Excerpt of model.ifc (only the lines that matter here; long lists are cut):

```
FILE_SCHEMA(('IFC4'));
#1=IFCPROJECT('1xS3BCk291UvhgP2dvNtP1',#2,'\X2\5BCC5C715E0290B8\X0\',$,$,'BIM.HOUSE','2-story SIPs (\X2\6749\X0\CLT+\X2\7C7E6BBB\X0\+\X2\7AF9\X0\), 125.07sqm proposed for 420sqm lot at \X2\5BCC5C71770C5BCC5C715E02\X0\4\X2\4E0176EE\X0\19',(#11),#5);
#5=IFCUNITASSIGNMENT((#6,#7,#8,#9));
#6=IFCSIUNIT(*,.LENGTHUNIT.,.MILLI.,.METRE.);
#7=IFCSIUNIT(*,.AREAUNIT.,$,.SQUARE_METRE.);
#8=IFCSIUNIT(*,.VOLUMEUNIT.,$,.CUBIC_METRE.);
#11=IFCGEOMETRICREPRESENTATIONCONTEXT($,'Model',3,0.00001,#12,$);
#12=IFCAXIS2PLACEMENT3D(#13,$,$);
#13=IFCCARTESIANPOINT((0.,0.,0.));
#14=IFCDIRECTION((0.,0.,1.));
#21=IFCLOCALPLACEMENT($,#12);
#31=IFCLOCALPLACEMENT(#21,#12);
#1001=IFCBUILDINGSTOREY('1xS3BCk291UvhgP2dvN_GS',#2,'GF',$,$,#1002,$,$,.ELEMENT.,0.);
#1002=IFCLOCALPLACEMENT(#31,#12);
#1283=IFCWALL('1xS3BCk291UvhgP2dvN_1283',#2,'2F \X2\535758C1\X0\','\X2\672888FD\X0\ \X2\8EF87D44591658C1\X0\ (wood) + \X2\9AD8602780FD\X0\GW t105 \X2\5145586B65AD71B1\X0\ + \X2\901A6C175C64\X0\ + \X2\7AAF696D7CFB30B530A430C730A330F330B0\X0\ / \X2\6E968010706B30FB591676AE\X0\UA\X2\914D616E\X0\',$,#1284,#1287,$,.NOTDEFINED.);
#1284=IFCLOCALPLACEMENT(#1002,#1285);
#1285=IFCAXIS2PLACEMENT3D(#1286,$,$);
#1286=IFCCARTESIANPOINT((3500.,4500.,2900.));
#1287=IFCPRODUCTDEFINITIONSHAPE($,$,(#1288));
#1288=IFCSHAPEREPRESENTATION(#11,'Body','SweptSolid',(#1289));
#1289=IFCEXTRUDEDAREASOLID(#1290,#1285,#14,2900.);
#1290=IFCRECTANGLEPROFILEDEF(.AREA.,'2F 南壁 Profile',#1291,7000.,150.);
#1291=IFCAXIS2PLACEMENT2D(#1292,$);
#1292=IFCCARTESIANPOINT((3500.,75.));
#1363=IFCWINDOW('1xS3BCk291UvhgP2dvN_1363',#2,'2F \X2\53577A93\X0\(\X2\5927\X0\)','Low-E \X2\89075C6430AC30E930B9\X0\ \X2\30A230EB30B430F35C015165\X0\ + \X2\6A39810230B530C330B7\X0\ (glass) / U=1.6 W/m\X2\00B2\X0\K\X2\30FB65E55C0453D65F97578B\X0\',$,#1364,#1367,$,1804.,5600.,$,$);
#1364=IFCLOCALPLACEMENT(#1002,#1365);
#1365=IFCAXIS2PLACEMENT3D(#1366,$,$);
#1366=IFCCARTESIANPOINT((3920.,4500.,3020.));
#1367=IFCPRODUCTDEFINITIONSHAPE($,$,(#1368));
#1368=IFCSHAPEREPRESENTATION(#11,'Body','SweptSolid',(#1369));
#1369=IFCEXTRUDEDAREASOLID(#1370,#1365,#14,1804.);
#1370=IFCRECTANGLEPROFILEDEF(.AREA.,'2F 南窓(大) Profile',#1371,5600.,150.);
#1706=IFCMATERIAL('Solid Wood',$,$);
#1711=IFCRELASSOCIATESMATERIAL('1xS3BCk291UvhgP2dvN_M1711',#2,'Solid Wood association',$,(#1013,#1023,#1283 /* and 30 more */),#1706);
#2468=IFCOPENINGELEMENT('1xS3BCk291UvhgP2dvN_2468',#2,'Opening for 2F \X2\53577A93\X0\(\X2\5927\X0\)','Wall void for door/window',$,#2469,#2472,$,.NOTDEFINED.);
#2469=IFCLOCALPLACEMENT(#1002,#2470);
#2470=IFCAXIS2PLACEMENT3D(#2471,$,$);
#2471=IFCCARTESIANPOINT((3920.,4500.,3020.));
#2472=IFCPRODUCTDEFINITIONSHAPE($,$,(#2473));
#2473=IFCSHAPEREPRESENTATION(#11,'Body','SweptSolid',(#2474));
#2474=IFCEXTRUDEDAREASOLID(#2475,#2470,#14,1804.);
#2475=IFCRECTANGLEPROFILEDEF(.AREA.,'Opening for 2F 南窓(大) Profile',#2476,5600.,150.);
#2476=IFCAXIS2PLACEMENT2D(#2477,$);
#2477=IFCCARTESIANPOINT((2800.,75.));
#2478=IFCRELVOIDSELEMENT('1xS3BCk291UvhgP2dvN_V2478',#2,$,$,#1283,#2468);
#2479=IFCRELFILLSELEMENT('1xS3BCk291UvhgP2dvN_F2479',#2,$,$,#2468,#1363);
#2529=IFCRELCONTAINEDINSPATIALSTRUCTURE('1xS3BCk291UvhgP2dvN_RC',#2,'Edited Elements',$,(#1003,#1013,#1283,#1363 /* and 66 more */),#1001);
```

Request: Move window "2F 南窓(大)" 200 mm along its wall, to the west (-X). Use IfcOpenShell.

```python
import ifcopenshell
import ifcopenshell.api.geometry
import ifcopenshell.util.placement
import ifcopenshell.util.unit

model = ifcopenshell.open("model.ifc")
unit_scale = ifcopenshell.util.unit.calculate_unit_scale(model)

window = model.by_guid("1xS3BCk291UvhgP2dvN_1363")
opening = window.FillsVoids[0].RelatingOpeningElement
wall = opening.VoidsElements[0].RelatingBuildingElement

wall_matrix = ifcopenshell.util.placement.get_local_placement(wall.ObjectPlacement)
shift = wall_matrix[:3, 0] * -0.2 / unit_scale
before = ifcopenshell.util.placement.get_local_placement(window.ObjectPlacement)[:3, 3].copy()

# The window is not placed relative to its opening, so move both.
for product in (opening, window):
    matrix = ifcopenshell.util.placement.get_local_placement(product.ObjectPlacement)
    matrix[:3, 3] += shift
    ifcopenshell.api.geometry.edit_object_placement(model, product=product, matrix=matrix, is_si=False)

after = ifcopenshell.util.placement.get_local_placement(window.ObjectPlacement)[:3, 3]
print("window moved by", (after - before).round(3) + 0.0)

model.write("model_updated.ifc")
```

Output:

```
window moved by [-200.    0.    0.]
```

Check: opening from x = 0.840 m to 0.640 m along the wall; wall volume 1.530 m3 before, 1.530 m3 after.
